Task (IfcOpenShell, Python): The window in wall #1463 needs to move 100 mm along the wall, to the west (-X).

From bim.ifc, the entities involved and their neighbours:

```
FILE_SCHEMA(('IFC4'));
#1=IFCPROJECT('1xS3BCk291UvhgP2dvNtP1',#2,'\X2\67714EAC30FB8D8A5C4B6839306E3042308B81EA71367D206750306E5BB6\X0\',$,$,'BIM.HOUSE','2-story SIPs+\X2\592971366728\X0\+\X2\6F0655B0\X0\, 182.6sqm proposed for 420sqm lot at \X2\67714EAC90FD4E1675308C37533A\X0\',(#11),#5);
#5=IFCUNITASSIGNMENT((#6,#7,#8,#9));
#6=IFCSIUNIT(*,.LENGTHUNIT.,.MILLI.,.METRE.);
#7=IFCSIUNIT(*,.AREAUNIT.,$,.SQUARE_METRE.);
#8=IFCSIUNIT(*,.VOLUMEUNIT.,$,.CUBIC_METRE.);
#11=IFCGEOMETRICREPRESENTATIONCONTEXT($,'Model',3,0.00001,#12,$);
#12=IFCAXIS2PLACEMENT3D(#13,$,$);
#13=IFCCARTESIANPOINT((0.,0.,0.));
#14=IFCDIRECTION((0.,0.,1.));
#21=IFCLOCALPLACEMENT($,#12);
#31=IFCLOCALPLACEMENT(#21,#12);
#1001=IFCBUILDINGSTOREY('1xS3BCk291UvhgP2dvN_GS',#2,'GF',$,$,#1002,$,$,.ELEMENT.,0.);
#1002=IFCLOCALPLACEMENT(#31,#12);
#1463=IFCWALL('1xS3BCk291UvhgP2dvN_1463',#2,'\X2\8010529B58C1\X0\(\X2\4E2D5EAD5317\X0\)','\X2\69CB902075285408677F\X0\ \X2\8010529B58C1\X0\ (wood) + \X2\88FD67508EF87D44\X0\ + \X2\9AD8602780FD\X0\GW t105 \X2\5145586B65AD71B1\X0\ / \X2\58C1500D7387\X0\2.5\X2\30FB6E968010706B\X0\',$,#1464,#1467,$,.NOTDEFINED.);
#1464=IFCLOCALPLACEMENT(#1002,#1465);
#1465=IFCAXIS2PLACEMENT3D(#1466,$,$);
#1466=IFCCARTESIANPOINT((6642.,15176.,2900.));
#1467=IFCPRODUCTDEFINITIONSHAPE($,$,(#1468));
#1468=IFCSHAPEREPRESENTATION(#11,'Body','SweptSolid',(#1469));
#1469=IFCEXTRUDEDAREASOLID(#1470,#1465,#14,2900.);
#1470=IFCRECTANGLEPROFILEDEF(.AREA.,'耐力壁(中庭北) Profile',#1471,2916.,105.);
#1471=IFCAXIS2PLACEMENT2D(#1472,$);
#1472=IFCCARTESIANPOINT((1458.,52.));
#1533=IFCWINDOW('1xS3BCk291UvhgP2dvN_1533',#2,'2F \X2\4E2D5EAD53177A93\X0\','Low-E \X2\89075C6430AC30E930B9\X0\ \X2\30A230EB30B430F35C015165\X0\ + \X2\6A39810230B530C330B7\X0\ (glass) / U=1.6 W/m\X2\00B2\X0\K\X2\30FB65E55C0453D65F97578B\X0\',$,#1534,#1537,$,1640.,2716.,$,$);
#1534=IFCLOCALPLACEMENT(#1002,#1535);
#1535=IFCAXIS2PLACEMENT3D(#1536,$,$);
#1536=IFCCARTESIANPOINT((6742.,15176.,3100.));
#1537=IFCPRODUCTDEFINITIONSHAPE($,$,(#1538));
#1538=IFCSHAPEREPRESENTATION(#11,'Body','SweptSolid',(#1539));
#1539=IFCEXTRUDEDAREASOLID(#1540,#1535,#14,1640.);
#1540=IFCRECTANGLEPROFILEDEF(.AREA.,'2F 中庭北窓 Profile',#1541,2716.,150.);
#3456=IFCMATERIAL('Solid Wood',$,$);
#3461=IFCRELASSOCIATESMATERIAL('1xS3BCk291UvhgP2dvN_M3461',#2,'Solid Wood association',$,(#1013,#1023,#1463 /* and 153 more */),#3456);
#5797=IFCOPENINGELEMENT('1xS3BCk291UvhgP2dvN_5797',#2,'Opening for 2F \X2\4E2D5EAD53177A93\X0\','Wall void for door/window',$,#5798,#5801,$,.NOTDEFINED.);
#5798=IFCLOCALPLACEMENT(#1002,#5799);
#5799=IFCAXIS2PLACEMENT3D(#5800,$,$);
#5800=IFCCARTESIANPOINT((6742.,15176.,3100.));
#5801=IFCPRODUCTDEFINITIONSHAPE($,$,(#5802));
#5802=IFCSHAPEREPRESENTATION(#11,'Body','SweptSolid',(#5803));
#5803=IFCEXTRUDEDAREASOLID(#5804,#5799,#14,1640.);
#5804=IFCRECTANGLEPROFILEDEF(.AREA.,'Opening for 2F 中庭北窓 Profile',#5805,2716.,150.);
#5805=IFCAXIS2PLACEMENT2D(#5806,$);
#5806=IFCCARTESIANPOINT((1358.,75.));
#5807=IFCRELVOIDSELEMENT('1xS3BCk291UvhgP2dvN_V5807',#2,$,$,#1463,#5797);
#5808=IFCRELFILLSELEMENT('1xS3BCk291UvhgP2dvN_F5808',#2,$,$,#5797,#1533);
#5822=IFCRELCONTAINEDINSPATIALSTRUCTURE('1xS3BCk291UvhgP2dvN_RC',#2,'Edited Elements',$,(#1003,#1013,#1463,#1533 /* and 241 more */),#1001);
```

```python
import ifcopenshell
import ifcopenshell.api.geometry
import ifcopenshell.util.placement
import ifcopenshell.util.unit

model = ifcopenshell.open("bim.ifc")
unit_scale = ifcopenshell.util.unit.calculate_unit_scale(model)

window = model.by_id(1533)
opening = window.FillsVoids[0].RelatingOpeningElement
wall = opening.VoidsElements[0].RelatingBuildingElement

wall_matrix = ifcopenshell.util.placement.get_local_placement(wall.ObjectPlacement)
shift = wall_matrix[:3, 0] * -0.1 / unit_scale
before = ifcopenshell.util.placement.get_local_placement(window.ObjectPlacement)[:3, 3].copy()

# The window is not placed relative to its opening, so move both.
for product in (opening, window):
    matrix = ifcopenshell.util.placement.get_local_placement(product.ObjectPlacement)
    matrix[:3, 3] += shift
    ifcopenshell.api.geometry.edit_object_placement(model, product=product, matrix=matrix, is_si=False)

after = ifcopenshell.util.placement.get_local_placement(window.ObjectPlacement)[:3, 3]
print("window moved by", (after - before).round(3) + 0.0)

model.write("bim-out.ifc")
```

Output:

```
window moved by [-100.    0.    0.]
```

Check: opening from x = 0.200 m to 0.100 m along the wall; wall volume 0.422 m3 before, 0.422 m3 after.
